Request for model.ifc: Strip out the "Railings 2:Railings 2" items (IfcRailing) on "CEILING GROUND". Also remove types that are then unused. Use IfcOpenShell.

First a look at what the model holds.

```python
import ifcopenshell
import ifcopenshell.util.element

model = ifcopenshell.open("model.ifc")
print(model.schema)
storey = next(s for s in model.by_type("IfcBuildingStorey") if s.Name == "CEILING GROUND")
railings = [e for e in ifcopenshell.util.element.get_decomposition(storey) if e.is_a("IfcRailing")]
seen = {}
for e in railings:
    element_type = ifcopenshell.util.element.get_type(e)
    name = element_type.Name if element_type not in (None, e) else None
    seen[name] = seen.get(name, 0) + 1
for name, count in sorted(seen.items(), key=str):
    print(count, "x", name)
```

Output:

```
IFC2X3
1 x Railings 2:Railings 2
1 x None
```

```python
import ifcopenshell
import ifcopenshell.api.root
import ifcopenshell.util.element

model = ifcopenshell.open("model.ifc")

storey = next(s for s in model.by_type("IfcBuildingStorey") if s.Name == "CEILING GROUND")
railings = [e for e in ifcopenshell.util.element.get_decomposition(storey) if e.is_a("IfcRailing")]
targets = [e for e in railings if (t := ifcopenshell.util.element.get_type(e)) not in (None, e) and t.Name == "Railings 2:Railings 2"]
types = {ifcopenshell.util.element.get_type(e) for e in targets} - {None, *targets}

for e in targets:
    ifcopenshell.api.root.remove_product(model, product=e)
print(len(targets), "removed")

unused = [t for t in types if not ifcopenshell.util.element.get_types(t)]
for t in unused:
    ifcopenshell.api.root.remove_product(model, product=t)
print(len(unused), "unused types removed")

model.write("model_rev.ifc")
```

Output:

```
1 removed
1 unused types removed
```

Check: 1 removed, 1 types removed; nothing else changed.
